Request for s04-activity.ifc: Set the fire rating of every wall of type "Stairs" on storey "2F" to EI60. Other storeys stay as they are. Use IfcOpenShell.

First a look at what the model holds.

```python
import ifcopenshell
import ifcopenshell.util.element

model = ifcopenshell.open("s04-activity.ifc")
print(model.schema)
storey = next(s for s in model.by_type("IfcBuildingStorey") if s.Name == "2F")
walls = [e for e in ifcopenshell.util.element.get_decomposition(storey) if e.is_a("IfcWall")]
seen = {}
for e in walls:
    element_type = ifcopenshell.util.element.get_type(e)
    key = (element_type.Name if element_type != e and element_type else None, ifcopenshell.util.element.get_pset(e, "Pset_WallCommon", "FireRating"))
    seen[key] = seen.get(key, 0) + 1
for (name, value), count in sorted(seen.items(), key=str):
    print(count, "x", name, "|", value)
```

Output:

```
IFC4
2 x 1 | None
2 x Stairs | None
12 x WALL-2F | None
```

```python
import ifcopenshell
import ifcopenshell.api.pset
import ifcopenshell.util.element

model = ifcopenshell.open("s04-activity.ifc")

storey = next(s for s in model.by_type("IfcBuildingStorey") if s.Name == "2F")
walls = [e for e in ifcopenshell.util.element.get_decomposition(storey) if e.is_a("IfcWall")]

count = 0
for e in walls:
    element_type = ifcopenshell.util.element.get_type(e)
    if element_type in (None, e) or element_type.Name != "Stairs":
        continue
    # add_pset returns the element's existing set when there is one.
    pset = ifcopenshell.api.pset.add_pset(model, product=e, name="Pset_WallCommon")
    ifcopenshell.api.pset.edit_pset(model, pset=pset, properties={"FireRating": "EI60"})
    count += 1

print(count, "walls updated")

model.write("s04-activity_rev.ifc")
```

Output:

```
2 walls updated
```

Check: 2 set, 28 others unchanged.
